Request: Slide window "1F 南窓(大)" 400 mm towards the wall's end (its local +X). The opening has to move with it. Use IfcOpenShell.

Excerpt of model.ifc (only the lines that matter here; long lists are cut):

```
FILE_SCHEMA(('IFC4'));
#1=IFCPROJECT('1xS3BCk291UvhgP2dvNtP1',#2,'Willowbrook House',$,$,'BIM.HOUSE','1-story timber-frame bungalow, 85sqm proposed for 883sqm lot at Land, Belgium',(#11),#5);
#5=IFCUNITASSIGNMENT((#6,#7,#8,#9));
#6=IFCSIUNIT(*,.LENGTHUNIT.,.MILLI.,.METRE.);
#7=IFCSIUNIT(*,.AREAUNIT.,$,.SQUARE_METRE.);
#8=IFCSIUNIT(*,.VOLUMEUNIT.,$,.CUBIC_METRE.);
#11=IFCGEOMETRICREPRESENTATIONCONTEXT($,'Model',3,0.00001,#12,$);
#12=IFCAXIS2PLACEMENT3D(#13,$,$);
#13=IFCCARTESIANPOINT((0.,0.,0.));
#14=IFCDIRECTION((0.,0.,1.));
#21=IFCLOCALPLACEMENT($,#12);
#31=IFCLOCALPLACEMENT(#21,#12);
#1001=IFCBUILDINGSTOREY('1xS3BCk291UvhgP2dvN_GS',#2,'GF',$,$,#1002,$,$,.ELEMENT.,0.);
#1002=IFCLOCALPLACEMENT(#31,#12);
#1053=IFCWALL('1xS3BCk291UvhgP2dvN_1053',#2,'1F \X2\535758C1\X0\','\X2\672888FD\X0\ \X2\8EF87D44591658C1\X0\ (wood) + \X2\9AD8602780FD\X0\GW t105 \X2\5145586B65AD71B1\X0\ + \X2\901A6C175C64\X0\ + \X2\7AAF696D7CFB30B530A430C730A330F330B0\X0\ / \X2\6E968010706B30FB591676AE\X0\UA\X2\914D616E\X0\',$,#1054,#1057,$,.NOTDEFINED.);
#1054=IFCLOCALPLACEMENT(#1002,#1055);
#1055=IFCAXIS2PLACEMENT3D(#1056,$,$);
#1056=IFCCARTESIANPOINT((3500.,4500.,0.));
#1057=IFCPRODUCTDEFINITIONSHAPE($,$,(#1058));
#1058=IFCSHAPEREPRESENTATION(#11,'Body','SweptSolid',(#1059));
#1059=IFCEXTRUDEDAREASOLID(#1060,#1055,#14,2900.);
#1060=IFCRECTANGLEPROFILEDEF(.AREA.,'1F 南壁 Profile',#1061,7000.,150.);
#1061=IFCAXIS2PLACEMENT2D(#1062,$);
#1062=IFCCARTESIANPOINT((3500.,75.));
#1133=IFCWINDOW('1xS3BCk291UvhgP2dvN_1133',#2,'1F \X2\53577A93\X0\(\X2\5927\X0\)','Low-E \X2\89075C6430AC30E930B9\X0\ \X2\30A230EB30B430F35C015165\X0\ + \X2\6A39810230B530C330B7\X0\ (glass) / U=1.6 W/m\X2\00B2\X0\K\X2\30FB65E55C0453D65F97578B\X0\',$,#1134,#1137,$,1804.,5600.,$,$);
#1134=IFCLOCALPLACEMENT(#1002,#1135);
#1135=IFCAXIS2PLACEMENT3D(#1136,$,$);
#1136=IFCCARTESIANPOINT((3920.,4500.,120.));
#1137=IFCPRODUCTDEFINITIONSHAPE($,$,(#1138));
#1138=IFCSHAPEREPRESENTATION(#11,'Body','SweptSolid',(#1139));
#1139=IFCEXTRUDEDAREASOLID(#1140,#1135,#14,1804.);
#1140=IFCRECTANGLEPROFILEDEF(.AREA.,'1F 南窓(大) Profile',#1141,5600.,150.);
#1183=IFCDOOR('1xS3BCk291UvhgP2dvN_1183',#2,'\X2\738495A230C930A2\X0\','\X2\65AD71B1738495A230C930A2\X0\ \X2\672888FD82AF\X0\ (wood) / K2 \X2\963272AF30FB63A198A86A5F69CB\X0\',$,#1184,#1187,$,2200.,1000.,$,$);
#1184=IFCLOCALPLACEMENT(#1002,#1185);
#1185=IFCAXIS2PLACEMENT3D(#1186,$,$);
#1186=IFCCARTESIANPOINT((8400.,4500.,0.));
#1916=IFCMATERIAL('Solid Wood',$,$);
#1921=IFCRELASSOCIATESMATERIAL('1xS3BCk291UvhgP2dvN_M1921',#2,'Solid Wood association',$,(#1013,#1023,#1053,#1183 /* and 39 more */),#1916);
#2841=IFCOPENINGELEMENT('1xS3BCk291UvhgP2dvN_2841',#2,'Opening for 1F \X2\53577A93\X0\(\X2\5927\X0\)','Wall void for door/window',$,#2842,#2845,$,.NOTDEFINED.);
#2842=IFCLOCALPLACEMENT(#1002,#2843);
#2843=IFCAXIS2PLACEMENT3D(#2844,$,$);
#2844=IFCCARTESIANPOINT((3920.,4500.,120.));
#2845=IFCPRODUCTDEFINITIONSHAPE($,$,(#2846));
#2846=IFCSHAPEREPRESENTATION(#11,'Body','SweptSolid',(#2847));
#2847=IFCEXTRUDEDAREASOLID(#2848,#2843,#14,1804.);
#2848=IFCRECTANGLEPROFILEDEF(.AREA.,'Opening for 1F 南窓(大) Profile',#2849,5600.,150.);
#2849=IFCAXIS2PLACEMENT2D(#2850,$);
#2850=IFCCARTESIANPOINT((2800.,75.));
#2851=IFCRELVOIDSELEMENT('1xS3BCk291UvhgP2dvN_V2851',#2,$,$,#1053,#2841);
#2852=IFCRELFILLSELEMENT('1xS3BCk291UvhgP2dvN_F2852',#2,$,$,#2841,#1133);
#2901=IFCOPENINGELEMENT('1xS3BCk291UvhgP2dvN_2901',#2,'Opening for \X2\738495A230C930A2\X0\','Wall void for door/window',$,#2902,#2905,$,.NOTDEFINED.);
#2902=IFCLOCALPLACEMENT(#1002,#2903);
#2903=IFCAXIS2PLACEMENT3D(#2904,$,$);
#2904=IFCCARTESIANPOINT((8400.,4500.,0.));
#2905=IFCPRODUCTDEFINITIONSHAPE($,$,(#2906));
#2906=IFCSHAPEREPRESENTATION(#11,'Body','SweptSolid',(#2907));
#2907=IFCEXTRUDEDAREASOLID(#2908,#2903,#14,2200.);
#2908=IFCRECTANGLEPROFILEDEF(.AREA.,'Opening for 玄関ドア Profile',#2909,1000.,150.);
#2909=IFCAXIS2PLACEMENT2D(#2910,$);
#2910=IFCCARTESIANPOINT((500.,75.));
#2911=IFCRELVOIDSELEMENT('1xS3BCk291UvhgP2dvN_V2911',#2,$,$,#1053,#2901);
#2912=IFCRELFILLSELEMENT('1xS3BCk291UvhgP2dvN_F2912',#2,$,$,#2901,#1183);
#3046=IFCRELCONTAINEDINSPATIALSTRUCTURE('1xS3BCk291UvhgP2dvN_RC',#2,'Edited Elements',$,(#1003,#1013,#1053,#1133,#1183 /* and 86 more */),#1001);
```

```python
import ifcopenshell
import ifcopenshell.api.geometry
import ifcopenshell.util.placement
import ifcopenshell.util.unit

model = ifcopenshell.open("model.ifc")
unit_scale = ifcopenshell.util.unit.calculate_unit_scale(model)

window = model.by_id(1133)
opening = window.FillsVoids[0].RelatingOpeningElement
wall = opening.VoidsElements[0].RelatingBuildingElement

wall_matrix = ifcopenshell.util.placement.get_local_placement(wall.ObjectPlacement)
shift = wall_matrix[:3, 0] * 0.4 / unit_scale
before = ifcopenshell.util.placement.get_local_placement(window.ObjectPlacement)[:3, 3].copy()

# The window is not placed relative to its opening, so move both.
for product in (opening, window):
    matrix = ifcopenshell.util.placement.get_local_placement(product.ObjectPlacement)
    matrix[:3, 3] += shift
    ifcopenshell.api.geometry.edit_object_placement(model, product=product, matrix=matrix, is_si=False)

after = ifcopenshell.util.placement.get_local_placement(window.ObjectPlacement)[:3, 3]
print("window moved by", (after - before).round(3) + 0.0)

model.write("model_v2.ifc")
```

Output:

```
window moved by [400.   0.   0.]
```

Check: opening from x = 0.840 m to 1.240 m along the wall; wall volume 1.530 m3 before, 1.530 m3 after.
